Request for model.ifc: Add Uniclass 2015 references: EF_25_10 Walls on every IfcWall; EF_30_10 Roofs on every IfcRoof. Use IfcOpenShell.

First a look at what the model holds.

```python
import ifcopenshell

model = ifcopenshell.open("model.ifc")
print(model.schema)
print("classifications:", [c.Name for c in model.by_type("IfcClassification")])
for ifc_class in ("IfcDoor", "IfcRoof", "IfcStair", "IfcWall", "IfcWindow"):
    print(ifc_class, len(model.by_type(ifc_class)))
```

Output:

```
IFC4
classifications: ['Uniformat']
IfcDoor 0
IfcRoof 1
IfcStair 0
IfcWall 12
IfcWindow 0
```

```python
import ifcopenshell
import ifcopenshell.api.classification

model = ifcopenshell.open("model.ifc")

system = ifcopenshell.api.classification.add_classification(model, classification="Uniclass 2015")

codes = {
    "IfcWall": ("EF_25_10", "Walls"),
    "IfcRoof": ("EF_30_10", "Roofs"),
}
for ifc_class, (code, name) in codes.items():
    products = model.by_type(ifc_class)
    ifcopenshell.api.classification.add_reference(
        model, products=products, classification=system, identification=code, name=name
    )
    print(code, len(products))

model.write("model_v2.ifc")
```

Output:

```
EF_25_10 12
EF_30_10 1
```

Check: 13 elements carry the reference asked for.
